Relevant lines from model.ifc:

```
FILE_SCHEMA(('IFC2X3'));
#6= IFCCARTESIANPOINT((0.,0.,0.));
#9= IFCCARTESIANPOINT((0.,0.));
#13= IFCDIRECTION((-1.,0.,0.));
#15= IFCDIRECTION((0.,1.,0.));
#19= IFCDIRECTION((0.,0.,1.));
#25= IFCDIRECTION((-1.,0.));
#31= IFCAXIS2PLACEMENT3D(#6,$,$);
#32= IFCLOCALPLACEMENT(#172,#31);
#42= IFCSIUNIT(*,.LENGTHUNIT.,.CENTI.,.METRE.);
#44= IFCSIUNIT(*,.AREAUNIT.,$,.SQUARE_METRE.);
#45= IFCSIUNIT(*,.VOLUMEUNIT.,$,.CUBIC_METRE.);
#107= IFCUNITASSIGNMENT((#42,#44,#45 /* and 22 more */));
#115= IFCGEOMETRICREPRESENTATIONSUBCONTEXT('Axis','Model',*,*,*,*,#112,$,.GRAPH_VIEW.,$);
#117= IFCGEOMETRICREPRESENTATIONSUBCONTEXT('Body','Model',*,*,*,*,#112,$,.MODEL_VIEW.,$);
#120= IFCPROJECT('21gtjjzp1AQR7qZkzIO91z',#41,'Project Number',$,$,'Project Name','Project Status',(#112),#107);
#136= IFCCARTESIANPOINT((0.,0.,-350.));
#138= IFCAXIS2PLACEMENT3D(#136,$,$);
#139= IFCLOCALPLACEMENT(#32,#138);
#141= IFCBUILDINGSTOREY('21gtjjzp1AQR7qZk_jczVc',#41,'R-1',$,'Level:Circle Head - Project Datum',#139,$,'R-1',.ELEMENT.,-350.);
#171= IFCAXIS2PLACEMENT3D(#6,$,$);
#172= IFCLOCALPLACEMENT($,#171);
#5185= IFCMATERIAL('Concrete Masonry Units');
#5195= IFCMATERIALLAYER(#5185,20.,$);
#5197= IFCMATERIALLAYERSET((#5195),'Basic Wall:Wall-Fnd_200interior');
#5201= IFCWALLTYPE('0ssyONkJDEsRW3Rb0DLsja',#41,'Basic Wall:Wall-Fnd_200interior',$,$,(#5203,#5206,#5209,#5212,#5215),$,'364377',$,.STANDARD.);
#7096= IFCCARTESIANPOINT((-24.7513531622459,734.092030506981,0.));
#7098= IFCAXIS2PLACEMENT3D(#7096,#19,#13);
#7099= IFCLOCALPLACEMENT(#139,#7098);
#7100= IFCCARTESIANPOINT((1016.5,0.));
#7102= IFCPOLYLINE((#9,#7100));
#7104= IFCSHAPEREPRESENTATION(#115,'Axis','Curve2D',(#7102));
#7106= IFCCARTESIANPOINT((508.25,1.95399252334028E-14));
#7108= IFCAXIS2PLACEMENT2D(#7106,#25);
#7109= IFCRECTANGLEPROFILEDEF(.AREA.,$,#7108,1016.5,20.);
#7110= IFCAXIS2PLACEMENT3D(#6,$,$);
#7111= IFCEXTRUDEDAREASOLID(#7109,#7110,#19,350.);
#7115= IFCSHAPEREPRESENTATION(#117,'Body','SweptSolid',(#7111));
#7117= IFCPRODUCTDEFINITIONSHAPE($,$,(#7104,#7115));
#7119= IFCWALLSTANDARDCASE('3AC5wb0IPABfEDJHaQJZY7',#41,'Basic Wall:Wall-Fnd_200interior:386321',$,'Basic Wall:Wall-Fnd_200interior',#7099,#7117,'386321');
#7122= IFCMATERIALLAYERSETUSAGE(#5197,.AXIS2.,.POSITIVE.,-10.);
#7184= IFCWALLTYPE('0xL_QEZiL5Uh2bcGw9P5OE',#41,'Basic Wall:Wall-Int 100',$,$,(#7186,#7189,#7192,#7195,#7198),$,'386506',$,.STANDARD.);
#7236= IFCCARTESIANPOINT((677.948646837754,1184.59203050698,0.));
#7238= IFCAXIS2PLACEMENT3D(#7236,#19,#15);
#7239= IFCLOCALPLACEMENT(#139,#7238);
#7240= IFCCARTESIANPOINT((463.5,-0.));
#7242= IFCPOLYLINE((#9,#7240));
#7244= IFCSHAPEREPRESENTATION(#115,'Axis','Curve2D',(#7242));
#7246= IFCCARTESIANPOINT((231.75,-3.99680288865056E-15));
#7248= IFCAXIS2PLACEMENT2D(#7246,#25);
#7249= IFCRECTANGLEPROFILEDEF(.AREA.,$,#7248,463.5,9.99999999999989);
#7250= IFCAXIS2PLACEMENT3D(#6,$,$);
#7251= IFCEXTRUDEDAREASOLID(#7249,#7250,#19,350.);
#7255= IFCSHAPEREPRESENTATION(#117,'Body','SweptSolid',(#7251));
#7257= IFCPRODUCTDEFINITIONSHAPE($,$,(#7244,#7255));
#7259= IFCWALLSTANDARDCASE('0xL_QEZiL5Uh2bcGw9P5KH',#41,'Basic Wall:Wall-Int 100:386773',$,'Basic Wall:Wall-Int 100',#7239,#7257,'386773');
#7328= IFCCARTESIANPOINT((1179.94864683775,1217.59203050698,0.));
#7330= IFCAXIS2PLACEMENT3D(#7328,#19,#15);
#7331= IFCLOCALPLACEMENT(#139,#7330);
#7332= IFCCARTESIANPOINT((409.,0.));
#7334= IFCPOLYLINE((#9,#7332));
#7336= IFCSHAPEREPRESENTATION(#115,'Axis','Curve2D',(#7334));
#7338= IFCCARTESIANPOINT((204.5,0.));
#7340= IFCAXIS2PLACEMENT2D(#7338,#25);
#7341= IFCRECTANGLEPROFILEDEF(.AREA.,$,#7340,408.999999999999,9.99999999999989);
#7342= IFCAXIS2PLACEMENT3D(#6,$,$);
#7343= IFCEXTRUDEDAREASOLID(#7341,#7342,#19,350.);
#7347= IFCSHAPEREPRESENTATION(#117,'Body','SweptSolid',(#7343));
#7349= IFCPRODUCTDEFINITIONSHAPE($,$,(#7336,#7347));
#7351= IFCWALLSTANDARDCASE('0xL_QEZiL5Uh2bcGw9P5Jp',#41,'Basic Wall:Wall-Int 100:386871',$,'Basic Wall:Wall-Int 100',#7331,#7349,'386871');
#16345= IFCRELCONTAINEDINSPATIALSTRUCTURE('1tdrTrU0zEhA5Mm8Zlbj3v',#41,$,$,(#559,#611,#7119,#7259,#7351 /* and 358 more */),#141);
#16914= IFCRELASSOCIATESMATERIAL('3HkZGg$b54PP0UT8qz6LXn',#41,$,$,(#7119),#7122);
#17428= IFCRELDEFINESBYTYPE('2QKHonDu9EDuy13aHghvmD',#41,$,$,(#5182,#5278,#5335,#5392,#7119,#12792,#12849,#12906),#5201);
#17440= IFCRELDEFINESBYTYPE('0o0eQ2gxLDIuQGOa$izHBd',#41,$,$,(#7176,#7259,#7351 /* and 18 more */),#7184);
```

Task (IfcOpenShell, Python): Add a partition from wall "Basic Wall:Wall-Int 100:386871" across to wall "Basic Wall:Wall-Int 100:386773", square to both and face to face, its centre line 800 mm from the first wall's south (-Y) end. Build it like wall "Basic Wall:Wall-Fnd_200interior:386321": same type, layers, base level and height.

```python
import numpy as np
import ifcopenshell
import ifcopenshell.api.geometry
import ifcopenshell.api.material
import ifcopenshell.api.pset
import ifcopenshell.api.root
import ifcopenshell.api.spatial
import ifcopenshell.api.type
import ifcopenshell.geom
import ifcopenshell.util.element
import ifcopenshell.util.placement
import ifcopenshell.util.representation
import ifcopenshell.util.shape
import ifcopenshell.util.unit

model = ifcopenshell.open("model.ifc")
unit_scale = ifcopenshell.util.unit.calculate_unit_scale(model)
settings = ifcopenshell.geom.settings()
settings.set("use-world-coords", True)

start_wall = model.by_guid("0xL_QEZiL5Uh2bcGw9P5Jp")
end_wall = model.by_guid("0xL_QEZiL5Uh2bcGw9P5KH")
like = model.by_id(7119)
matrix = ifcopenshell.util.placement.get_local_placement(start_wall.ObjectPlacement)
matrix[:3, 3] *= unit_scale


def extent(element):
    """Bounding box in the first wall's axes, in metres."""
    shape = ifcopenshell.geom.create_shape(settings, element)
    points = (ifcopenshell.util.shape.get_vertices(shape.geometry) - matrix[:3, 3]) @ matrix[:3, :3]
    return points.min(axis=0), points.max(axis=0)


y_start = extent(start_wall)[1][1]
y_end = extent(end_wall)[0][1]
like_min, like_max = extent(like)
length, height = float(abs(y_end - y_start)), float(like_max[2] - like_min[2])
layer_set = ifcopenshell.util.element.get_material(like, should_skip_usage=True)
thickness = sum(layer.LayerThickness for layer in layer_set.MaterialLayers) * unit_scale

wall = ifcopenshell.api.root.create_entity(model, ifc_class="IfcWallStandardCase", name="New partition")
storey = ifcopenshell.util.element.get_container(like)
ifcopenshell.api.spatial.assign_container(model, products=[wall], relating_structure=storey)
ifcopenshell.api.type.assign_type(
    model, related_objects=[wall], relating_type=ifcopenshell.util.element.get_type(like), should_map_representations=False
)
rel = ifcopenshell.api.material.assign_material(
    model, products=[wall], type="IfcMaterialLayerSetUsage", material=layer_set
)
rel.RelatingMaterial.OffsetFromReferenceLine = -thickness / 2 / unit_scale
pset = ifcopenshell.api.pset.add_pset(model, product=wall, name="Pset_WallCommon")
ifcopenshell.api.pset.edit_pset(model, pset=pset, properties={"IsExternal": False, "LoadBearing": False})

# The axis runs down the middle of the wall.
axis = ifcopenshell.api.geometry.add_axis_representation(
    model, context=ifcopenshell.util.representation.get_context(model, "Model", "Axis"), axis=[(0.0, 0.0), (length, 0.0)]
)
body = ifcopenshell.api.geometry.add_wall_representation(
    model,
    context=ifcopenshell.util.representation.get_context(model, "Model", "Body", "MODEL_VIEW"),
    length=length,
    height=height,
    thickness=thickness,
    offset=-thickness / 2,
)
for representation in (axis, body):
    ifcopenshell.api.geometry.assign_representation(model, product=wall, representation=representation)

placement = matrix @ ifcopenshell.util.placement.rotation(90, "Z")
placement[:, 3] = matrix @ np.array([extent(start_wall)[0][0] + 0.8, y_start, like_min[2], 1.0])
ifcopenshell.api.geometry.edit_object_placement(model, product=wall, matrix=placement)

print(f"partition {length:.3f} m long, {height:.3f} m high, {thickness:.3f} m thick")

model.write("model_updated.ifc")
```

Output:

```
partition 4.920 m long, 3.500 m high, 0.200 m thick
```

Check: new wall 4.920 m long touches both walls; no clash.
